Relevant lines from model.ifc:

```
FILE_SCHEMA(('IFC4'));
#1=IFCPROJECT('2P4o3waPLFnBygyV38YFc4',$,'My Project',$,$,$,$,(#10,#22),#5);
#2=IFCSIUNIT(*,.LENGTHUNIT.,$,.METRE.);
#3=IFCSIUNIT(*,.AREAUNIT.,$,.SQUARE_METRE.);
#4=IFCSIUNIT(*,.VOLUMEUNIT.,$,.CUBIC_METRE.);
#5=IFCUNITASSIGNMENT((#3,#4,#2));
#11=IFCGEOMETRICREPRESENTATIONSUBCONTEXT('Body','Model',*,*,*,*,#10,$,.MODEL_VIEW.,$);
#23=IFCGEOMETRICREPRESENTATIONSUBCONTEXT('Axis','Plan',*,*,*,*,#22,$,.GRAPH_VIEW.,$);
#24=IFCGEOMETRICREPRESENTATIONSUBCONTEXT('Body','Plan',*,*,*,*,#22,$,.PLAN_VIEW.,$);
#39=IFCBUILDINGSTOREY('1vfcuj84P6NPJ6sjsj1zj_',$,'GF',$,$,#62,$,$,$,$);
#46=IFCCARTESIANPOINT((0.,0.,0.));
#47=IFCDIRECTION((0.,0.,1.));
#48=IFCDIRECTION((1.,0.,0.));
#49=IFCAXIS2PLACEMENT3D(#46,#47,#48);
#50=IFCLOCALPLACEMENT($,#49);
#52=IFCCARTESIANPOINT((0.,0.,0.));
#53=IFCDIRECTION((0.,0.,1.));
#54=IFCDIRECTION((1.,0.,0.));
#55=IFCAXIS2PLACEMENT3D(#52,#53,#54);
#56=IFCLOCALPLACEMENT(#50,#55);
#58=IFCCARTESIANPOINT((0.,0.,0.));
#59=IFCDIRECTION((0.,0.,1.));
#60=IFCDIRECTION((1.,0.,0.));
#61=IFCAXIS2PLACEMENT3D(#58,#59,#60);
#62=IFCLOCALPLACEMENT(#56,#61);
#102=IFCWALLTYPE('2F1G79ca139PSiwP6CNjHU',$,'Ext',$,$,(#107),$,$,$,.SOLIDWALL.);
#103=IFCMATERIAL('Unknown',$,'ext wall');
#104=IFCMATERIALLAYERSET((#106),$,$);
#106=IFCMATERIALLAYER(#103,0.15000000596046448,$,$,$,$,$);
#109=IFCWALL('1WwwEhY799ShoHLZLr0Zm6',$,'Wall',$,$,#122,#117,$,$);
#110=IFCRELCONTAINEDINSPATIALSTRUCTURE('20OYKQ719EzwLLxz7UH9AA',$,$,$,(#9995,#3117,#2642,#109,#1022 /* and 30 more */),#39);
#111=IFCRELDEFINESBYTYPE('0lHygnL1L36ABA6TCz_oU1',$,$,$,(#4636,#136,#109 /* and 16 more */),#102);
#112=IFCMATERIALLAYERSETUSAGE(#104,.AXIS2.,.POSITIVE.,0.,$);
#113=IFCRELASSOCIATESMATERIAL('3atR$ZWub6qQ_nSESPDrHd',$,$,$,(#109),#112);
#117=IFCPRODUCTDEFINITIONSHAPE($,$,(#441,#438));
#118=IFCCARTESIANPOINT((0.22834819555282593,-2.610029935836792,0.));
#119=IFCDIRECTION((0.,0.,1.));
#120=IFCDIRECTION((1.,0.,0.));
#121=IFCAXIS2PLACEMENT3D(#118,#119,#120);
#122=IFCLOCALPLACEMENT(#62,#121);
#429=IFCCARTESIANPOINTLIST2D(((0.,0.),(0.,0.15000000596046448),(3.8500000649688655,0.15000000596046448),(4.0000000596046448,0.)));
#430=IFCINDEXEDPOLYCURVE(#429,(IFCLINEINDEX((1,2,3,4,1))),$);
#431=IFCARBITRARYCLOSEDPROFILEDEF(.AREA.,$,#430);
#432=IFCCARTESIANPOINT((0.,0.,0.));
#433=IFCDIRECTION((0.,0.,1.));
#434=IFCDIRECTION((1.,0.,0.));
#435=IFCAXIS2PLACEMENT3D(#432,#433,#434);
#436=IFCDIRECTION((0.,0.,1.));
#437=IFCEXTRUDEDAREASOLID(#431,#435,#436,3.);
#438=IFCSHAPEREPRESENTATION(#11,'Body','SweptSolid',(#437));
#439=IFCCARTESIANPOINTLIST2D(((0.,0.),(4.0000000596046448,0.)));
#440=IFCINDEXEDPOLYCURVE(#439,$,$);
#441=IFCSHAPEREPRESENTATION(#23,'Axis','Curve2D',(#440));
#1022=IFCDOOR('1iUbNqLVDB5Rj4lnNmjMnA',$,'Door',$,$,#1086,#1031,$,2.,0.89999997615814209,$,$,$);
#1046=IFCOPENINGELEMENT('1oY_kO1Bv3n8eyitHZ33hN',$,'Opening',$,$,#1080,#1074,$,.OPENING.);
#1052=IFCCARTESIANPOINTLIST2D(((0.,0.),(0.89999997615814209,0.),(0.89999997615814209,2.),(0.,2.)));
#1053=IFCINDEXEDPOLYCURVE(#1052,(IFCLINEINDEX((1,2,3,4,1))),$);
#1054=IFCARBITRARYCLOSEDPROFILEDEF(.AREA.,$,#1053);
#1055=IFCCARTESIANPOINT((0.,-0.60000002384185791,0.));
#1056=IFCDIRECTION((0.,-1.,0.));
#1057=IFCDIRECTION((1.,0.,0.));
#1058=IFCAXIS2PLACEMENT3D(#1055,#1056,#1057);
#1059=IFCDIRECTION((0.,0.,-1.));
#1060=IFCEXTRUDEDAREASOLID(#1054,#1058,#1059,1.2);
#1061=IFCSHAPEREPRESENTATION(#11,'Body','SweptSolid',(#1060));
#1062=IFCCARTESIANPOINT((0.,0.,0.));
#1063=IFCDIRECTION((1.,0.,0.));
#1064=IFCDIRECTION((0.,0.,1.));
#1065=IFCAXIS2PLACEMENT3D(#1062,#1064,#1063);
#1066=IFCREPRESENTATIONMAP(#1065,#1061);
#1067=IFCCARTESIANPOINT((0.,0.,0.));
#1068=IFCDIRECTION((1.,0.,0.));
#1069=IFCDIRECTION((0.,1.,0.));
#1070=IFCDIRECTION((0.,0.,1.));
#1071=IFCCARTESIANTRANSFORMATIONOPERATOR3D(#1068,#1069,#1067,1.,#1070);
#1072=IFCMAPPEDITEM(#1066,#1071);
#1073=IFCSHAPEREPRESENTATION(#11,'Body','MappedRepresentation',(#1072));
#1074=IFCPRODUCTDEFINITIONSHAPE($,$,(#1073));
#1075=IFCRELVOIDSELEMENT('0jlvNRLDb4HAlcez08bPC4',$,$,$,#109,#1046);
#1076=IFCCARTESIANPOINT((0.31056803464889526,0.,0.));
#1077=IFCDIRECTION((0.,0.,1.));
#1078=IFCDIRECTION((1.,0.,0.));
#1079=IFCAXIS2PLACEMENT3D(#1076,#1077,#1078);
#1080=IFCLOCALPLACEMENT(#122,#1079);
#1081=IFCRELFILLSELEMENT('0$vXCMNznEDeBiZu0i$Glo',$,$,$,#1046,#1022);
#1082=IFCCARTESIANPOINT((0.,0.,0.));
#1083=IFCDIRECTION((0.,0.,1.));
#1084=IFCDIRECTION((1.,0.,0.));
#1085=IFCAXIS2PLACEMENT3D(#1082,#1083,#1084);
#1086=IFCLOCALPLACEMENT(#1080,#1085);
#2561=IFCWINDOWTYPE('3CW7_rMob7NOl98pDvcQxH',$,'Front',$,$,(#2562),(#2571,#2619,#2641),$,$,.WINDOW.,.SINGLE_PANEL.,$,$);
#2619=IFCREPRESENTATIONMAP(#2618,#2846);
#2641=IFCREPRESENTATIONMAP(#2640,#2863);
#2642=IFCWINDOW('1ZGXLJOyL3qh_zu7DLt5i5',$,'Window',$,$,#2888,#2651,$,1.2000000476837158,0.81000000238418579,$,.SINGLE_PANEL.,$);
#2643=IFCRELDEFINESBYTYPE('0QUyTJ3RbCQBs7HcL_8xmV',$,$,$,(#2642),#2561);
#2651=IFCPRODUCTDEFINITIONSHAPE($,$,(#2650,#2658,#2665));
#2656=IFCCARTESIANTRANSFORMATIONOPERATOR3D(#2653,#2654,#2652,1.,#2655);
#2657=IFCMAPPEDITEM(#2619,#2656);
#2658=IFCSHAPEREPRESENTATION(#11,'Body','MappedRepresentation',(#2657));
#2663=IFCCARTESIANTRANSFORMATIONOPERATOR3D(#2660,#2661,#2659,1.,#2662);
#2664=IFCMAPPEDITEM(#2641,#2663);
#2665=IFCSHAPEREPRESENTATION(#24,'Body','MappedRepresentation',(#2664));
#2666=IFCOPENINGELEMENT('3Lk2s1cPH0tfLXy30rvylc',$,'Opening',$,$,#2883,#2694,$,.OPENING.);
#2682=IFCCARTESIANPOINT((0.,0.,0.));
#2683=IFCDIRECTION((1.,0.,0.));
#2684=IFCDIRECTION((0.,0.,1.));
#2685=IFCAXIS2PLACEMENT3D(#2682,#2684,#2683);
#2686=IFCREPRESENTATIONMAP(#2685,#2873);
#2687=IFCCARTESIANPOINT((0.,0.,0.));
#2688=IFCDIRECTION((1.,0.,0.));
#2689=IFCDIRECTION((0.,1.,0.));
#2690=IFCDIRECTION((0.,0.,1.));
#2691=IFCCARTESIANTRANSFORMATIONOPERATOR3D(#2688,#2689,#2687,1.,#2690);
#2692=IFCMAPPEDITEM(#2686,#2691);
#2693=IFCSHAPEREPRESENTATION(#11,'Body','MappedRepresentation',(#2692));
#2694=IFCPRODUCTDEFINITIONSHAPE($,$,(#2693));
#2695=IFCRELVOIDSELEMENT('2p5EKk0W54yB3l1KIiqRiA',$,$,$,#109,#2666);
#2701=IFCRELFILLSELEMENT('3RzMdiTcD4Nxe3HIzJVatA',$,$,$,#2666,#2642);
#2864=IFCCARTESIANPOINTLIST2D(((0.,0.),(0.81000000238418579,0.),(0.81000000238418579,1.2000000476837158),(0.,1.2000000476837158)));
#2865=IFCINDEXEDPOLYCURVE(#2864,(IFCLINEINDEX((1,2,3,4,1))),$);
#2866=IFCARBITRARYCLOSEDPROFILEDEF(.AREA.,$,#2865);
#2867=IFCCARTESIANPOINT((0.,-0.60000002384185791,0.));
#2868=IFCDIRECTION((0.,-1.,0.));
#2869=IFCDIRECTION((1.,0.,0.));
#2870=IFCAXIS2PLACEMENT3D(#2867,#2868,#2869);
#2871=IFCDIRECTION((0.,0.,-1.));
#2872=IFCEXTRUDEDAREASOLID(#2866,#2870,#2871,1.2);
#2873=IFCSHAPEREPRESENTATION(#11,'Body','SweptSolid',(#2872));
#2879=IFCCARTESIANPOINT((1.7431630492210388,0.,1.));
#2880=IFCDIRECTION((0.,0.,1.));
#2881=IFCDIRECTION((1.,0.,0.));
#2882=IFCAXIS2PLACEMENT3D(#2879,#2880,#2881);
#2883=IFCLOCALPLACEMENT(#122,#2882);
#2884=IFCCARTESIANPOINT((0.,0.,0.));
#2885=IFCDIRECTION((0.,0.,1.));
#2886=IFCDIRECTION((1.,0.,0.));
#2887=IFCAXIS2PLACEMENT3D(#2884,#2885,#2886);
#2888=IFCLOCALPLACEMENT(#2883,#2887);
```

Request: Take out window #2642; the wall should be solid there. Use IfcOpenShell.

```python
import ifcopenshell
import ifcopenshell.api.feature
import ifcopenshell.api.root
import ifcopenshell.geom
import ifcopenshell.util.shape

model = ifcopenshell.open("model.ifc")
settings = ifcopenshell.geom.settings()


def volume(element):
    """Net volume in cubic metres, openings subtracted."""
    shape = ifcopenshell.geom.create_shape(settings, element)
    return ifcopenshell.util.shape.get_volume(shape.geometry)


window = model.by_guid("1ZGXLJOyL3qh_zu7DLt5i5")
opening = window.FillsVoids[0].RelatingOpeningElement
wall = opening.VoidsElements[0].RelatingBuildingElement
before = volume(wall)

ifcopenshell.api.root.remove_product(model, product=window)
ifcopenshell.api.feature.remove_feature(model, feature=opening)

after = volume(wall)

print(f"wall volume {before:.3f} -> {after:.3f} m3")

model.write("model-out.ifc")
```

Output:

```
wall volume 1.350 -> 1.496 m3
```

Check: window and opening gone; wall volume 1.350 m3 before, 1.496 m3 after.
